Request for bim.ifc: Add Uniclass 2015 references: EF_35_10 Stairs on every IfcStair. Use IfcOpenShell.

First a look at what the model holds.

```python
import ifcopenshell

model = ifcopenshell.open("bim.ifc")
print(model.schema)
print("classifications:", [c.Name for c in model.by_type("IfcClassification")])
for ifc_class in ("IfcDoor", "IfcRoof", "IfcStair", "IfcWall", "IfcWindow"):
    print(ifc_class, len(model.by_type(ifc_class)))
```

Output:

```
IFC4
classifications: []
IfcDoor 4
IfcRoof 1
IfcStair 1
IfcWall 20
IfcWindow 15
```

```python
import ifcopenshell
import ifcopenshell.api.classification

model = ifcopenshell.open("bim.ifc")

system = ifcopenshell.api.classification.add_classification(model, classification="Uniclass 2015")

codes = {
    "IfcStair": ("EF_35_10", "Stairs"),
}
for ifc_class, (code, name) in codes.items():
    products = model.by_type(ifc_class)
    ifcopenshell.api.classification.add_reference(
        model, products=products, classification=system, identification=code, name=name
    )
    print(code, len(products))

model.write("bim-out.ifc")
```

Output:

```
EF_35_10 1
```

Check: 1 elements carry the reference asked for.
